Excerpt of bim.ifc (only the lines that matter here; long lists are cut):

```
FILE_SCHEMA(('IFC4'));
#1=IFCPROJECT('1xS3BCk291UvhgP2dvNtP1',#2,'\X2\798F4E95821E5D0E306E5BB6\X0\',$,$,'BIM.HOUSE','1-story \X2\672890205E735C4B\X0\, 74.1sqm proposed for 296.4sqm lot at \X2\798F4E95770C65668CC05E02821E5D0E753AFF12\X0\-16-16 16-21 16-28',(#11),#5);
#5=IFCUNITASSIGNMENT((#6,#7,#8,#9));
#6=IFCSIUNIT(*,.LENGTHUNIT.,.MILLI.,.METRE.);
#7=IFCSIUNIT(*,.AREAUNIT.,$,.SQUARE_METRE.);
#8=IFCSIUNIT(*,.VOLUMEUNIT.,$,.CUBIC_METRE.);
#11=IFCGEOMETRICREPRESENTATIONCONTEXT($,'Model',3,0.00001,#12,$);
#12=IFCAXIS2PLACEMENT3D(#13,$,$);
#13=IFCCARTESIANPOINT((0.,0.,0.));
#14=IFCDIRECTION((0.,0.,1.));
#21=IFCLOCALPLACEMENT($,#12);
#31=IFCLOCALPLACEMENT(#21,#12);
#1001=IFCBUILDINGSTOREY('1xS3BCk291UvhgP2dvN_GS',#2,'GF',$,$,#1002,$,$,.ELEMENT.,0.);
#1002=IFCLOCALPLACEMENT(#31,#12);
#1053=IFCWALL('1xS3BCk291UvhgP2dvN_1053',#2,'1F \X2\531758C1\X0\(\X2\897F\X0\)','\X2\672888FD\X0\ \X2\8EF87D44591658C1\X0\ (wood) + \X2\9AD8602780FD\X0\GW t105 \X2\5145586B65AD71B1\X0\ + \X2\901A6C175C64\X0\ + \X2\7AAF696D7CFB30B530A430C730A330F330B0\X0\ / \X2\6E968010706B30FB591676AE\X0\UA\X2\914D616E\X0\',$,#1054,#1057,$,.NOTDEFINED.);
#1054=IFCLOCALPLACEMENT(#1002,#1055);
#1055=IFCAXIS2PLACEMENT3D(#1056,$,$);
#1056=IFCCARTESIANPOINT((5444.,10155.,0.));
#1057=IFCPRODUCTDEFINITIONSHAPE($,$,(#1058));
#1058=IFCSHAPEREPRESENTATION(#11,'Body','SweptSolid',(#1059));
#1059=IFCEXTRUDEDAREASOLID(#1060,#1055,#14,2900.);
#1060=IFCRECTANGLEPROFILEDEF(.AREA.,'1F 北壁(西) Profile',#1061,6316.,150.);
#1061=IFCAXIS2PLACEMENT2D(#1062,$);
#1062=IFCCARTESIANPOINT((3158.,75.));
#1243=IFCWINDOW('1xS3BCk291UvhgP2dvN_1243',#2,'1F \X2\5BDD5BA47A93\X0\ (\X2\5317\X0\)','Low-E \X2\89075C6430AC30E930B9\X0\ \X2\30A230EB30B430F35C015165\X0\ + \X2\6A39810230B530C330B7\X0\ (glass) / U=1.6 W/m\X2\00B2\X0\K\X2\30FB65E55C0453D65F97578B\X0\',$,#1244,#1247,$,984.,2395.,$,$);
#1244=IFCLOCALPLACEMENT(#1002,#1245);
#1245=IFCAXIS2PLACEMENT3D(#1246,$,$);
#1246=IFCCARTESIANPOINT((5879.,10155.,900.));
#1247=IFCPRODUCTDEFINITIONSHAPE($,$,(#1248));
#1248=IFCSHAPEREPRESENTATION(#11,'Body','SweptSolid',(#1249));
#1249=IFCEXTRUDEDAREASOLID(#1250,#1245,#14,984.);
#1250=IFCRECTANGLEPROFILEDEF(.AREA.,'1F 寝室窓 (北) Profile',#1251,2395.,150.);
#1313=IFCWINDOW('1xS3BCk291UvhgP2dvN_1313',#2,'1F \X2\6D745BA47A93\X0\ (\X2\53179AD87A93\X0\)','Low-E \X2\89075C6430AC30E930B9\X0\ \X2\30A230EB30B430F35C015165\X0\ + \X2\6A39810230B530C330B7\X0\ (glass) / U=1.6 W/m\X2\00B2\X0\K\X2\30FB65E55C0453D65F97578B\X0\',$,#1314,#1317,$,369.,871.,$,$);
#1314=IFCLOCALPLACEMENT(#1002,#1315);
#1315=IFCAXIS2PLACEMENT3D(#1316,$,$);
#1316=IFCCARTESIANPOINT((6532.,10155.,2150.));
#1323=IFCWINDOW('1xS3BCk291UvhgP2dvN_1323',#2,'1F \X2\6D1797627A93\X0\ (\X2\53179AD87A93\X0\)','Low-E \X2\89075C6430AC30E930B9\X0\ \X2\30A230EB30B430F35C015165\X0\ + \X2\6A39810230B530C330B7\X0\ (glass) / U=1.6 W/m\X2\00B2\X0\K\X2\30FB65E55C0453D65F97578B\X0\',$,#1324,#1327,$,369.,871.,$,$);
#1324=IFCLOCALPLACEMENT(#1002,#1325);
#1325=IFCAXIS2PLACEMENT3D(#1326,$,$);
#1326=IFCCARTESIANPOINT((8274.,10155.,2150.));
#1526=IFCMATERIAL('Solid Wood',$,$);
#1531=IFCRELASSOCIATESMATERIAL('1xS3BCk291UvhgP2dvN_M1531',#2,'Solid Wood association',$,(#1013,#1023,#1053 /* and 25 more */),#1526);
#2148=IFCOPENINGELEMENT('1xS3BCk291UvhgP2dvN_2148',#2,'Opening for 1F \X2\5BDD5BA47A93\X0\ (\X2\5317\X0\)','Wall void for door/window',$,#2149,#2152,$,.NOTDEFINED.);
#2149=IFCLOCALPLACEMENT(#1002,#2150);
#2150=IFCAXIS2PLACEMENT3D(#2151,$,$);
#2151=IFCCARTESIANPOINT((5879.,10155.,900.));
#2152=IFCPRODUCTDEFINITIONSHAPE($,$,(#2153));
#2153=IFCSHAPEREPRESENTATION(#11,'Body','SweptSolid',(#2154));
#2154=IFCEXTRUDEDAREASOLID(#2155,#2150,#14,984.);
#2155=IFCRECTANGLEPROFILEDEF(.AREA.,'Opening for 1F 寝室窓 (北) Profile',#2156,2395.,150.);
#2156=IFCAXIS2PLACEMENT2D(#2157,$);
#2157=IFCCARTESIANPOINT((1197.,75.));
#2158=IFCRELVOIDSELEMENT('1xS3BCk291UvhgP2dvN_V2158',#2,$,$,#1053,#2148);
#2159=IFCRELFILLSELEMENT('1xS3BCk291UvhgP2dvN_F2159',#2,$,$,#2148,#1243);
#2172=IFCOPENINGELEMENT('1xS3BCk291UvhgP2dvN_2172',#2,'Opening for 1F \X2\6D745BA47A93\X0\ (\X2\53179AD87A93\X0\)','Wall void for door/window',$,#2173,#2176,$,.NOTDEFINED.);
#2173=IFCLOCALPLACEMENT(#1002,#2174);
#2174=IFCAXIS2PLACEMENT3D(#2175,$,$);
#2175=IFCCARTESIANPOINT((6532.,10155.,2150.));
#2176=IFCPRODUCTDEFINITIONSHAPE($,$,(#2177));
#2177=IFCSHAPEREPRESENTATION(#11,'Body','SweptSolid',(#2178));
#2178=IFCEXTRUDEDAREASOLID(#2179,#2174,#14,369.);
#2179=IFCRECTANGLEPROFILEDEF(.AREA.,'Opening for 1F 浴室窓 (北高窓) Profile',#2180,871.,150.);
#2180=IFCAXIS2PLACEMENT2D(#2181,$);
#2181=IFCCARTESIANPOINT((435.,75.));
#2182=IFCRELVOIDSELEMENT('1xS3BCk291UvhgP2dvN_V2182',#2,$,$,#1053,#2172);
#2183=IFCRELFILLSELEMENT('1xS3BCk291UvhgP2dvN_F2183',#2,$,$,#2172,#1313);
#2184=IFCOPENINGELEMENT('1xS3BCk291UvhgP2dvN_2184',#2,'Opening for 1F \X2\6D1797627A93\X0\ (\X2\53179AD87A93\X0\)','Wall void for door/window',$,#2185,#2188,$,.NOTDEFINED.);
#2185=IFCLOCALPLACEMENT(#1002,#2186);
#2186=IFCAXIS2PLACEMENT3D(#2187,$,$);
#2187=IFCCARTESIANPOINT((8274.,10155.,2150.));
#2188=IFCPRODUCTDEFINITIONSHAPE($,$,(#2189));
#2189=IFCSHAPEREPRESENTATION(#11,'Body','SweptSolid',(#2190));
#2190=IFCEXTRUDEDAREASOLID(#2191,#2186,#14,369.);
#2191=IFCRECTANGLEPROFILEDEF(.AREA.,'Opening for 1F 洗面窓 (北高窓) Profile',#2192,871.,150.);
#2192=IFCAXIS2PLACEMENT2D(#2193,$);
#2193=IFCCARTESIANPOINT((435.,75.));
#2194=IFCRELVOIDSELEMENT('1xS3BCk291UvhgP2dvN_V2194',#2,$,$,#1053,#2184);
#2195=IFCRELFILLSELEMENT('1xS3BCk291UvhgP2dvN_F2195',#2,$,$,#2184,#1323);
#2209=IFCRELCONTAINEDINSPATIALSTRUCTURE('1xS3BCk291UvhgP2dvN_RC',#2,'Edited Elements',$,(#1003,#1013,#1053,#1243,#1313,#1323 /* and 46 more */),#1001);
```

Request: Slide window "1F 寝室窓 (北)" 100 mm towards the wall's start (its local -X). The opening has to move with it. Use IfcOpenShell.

```python
import ifcopenshell
import ifcopenshell.api.geometry
import ifcopenshell.util.placement
import ifcopenshell.util.unit

model = ifcopenshell.open("bim.ifc")
unit_scale = ifcopenshell.util.unit.calculate_unit_scale(model)

window = model.by_id(1243)
opening = window.FillsVoids[0].RelatingOpeningElement
wall = opening.VoidsElements[0].RelatingBuildingElement

wall_matrix = ifcopenshell.util.placement.get_local_placement(wall.ObjectPlacement)
shift = wall_matrix[:3, 0] * -0.1 / unit_scale
before = ifcopenshell.util.placement.get_local_placement(window.ObjectPlacement)[:3, 3].copy()

# The window is not placed relative to its opening, so move both.
for product in (opening, window):
    matrix = ifcopenshell.util.placement.get_local_placement(product.ObjectPlacement)
    matrix[:3, 3] += shift
    ifcopenshell.api.geometry.edit_object_placement(model, product=product, matrix=matrix, is_si=False)

after = ifcopenshell.util.placement.get_local_placement(window.ObjectPlacement)[:3, 3]
print("window moved by", (after - before).round(3) + 0.0)

model.write("bim_rev.ifc")
```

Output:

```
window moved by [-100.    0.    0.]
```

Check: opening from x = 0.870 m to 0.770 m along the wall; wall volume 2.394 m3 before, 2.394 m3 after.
